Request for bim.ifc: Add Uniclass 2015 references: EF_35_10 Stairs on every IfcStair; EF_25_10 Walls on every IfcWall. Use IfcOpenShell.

First a look at what the model holds.

```python
import ifcopenshell

model = ifcopenshell.open("bim.ifc")
print(model.schema)
print("classifications:", [c.Name for c in model.by_type("IfcClassification")])
for ifc_class in ("IfcDoor", "IfcRoof", "IfcStair", "IfcWall", "IfcWindow"):
    print(ifc_class, len(model.by_type(ifc_class)))
```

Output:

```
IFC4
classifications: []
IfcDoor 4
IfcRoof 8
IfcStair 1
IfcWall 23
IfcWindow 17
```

```python
import ifcopenshell
import ifcopenshell.api.classification

model = ifcopenshell.open("bim.ifc")

system = ifcopenshell.api.classification.add_classification(model, classification="Uniclass 2015")

codes = {
    "IfcStair": ("EF_35_10", "Stairs"),
    "IfcWall": ("EF_25_10", "Walls"),
}
for ifc_class, (code, name) in codes.items():
    products = model.by_type(ifc_class)
    ifcopenshell.api.classification.add_reference(
        model, products=products, classification=system, identification=code, name=name
    )
    print(code, len(products))

model.write("bim_rev.ifc")
```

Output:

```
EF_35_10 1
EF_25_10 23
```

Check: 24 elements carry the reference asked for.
